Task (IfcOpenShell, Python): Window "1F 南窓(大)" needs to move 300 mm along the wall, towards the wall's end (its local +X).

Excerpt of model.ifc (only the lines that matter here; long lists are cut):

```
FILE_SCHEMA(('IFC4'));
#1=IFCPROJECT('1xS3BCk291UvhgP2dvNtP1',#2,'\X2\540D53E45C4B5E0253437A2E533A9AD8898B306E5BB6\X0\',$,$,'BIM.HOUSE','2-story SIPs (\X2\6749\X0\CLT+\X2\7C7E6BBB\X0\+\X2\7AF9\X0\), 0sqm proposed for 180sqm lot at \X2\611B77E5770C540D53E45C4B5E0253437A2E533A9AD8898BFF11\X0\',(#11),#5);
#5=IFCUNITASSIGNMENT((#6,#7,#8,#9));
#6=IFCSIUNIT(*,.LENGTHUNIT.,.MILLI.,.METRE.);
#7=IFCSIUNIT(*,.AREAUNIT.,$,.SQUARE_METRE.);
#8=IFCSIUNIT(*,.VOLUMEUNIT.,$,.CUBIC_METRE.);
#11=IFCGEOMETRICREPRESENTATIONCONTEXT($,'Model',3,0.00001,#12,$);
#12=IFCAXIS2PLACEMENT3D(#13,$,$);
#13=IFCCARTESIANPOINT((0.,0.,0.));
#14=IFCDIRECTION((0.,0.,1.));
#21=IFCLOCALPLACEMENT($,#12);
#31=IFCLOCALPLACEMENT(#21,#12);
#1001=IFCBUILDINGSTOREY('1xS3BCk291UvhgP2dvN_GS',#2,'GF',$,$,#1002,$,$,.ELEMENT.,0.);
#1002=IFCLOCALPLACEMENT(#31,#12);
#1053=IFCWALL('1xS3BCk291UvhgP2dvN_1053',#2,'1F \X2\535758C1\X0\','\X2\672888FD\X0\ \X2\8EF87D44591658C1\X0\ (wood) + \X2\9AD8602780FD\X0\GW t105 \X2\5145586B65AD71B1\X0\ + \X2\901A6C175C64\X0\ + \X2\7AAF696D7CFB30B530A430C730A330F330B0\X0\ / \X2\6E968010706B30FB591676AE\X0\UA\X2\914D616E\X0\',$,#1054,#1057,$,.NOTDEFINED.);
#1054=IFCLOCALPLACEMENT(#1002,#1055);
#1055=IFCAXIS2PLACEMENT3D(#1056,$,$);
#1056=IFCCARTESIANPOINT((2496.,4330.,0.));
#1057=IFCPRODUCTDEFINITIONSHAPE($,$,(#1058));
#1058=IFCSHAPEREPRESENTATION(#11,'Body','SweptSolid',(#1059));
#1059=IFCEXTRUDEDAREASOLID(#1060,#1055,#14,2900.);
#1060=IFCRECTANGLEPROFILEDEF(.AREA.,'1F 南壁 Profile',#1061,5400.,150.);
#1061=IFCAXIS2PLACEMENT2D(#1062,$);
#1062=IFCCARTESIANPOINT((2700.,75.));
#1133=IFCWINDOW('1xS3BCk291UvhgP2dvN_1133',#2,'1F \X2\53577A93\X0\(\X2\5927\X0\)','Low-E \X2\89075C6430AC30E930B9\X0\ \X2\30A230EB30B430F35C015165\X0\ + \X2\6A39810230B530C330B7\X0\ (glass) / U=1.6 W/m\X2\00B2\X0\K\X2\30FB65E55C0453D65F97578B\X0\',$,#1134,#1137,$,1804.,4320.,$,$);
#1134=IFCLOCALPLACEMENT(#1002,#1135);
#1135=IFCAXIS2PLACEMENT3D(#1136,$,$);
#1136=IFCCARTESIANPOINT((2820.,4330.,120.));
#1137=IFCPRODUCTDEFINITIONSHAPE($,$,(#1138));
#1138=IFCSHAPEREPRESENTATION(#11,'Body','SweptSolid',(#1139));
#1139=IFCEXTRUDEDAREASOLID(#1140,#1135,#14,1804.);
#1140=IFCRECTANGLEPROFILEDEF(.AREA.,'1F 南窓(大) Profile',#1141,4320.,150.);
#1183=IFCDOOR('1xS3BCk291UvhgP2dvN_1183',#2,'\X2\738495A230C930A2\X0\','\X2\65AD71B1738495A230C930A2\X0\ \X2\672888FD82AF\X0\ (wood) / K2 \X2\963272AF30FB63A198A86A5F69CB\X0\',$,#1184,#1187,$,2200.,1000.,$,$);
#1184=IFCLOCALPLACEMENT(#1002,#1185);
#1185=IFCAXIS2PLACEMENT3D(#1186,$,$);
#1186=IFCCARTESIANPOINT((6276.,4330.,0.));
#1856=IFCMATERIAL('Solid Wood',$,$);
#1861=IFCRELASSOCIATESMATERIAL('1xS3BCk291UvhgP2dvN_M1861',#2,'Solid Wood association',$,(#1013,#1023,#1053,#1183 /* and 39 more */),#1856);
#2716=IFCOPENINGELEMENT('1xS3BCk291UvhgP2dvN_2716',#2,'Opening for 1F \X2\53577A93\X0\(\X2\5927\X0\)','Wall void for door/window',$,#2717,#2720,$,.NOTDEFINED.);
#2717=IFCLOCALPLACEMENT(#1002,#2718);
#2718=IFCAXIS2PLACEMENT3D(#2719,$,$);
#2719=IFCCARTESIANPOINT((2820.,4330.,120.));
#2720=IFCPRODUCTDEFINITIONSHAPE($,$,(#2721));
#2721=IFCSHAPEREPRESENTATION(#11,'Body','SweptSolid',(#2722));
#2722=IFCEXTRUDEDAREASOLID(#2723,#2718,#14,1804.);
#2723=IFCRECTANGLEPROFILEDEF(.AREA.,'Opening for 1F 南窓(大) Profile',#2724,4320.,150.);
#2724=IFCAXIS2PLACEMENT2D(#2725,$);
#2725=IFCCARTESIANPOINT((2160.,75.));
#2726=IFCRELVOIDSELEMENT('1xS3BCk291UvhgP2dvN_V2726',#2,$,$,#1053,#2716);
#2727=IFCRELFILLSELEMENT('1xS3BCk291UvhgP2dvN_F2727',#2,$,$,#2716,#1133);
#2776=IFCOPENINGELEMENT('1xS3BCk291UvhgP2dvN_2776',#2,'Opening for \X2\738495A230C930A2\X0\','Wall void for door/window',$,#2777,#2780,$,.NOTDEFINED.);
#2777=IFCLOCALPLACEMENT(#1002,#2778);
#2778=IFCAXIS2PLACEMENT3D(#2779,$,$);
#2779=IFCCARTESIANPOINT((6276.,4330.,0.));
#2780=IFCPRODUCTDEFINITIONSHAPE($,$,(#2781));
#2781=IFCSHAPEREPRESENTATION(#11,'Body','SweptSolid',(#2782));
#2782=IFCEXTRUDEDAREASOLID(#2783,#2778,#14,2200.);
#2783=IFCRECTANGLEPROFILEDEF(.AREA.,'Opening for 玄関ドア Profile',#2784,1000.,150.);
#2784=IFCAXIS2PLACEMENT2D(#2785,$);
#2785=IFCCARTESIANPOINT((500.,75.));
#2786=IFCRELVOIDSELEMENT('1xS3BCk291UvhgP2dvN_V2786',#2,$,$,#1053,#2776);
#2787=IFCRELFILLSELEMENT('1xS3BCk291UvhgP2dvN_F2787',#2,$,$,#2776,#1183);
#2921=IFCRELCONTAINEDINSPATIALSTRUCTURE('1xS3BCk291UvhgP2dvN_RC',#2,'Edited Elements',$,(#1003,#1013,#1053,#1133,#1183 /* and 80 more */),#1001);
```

```python
import ifcopenshell
import ifcopenshell.api.geometry
import ifcopenshell.util.placement
import ifcopenshell.util.unit

model = ifcopenshell.open("model.ifc")
unit_scale = ifcopenshell.util.unit.calculate_unit_scale(model)

window = model.by_guid("1xS3BCk291UvhgP2dvN_1133")
opening = window.FillsVoids[0].RelatingOpeningElement
wall = opening.VoidsElements[0].RelatingBuildingElement

wall_matrix = ifcopenshell.util.placement.get_local_placement(wall.ObjectPlacement)
shift = wall_matrix[:3, 0] * 0.3 / unit_scale
before = ifcopenshell.util.placement.get_local_placement(window.ObjectPlacement)[:3, 3].copy()

# The window is not placed relative to its opening, so move both.
for product in (opening, window):
    matrix = ifcopenshell.util.placement.get_local_placement(product.ObjectPlacement)
    matrix[:3, 3] += shift
    ifcopenshell.api.geometry.edit_object_placement(model, product=product, matrix=matrix, is_si=False)

after = ifcopenshell.util.placement.get_local_placement(window.ObjectPlacement)[:3, 3]
print("window moved by", (after - before).round(3) + 0.0)

model.write("model_v2.ifc")
```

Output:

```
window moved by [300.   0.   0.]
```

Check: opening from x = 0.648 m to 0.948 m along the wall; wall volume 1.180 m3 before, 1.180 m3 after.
